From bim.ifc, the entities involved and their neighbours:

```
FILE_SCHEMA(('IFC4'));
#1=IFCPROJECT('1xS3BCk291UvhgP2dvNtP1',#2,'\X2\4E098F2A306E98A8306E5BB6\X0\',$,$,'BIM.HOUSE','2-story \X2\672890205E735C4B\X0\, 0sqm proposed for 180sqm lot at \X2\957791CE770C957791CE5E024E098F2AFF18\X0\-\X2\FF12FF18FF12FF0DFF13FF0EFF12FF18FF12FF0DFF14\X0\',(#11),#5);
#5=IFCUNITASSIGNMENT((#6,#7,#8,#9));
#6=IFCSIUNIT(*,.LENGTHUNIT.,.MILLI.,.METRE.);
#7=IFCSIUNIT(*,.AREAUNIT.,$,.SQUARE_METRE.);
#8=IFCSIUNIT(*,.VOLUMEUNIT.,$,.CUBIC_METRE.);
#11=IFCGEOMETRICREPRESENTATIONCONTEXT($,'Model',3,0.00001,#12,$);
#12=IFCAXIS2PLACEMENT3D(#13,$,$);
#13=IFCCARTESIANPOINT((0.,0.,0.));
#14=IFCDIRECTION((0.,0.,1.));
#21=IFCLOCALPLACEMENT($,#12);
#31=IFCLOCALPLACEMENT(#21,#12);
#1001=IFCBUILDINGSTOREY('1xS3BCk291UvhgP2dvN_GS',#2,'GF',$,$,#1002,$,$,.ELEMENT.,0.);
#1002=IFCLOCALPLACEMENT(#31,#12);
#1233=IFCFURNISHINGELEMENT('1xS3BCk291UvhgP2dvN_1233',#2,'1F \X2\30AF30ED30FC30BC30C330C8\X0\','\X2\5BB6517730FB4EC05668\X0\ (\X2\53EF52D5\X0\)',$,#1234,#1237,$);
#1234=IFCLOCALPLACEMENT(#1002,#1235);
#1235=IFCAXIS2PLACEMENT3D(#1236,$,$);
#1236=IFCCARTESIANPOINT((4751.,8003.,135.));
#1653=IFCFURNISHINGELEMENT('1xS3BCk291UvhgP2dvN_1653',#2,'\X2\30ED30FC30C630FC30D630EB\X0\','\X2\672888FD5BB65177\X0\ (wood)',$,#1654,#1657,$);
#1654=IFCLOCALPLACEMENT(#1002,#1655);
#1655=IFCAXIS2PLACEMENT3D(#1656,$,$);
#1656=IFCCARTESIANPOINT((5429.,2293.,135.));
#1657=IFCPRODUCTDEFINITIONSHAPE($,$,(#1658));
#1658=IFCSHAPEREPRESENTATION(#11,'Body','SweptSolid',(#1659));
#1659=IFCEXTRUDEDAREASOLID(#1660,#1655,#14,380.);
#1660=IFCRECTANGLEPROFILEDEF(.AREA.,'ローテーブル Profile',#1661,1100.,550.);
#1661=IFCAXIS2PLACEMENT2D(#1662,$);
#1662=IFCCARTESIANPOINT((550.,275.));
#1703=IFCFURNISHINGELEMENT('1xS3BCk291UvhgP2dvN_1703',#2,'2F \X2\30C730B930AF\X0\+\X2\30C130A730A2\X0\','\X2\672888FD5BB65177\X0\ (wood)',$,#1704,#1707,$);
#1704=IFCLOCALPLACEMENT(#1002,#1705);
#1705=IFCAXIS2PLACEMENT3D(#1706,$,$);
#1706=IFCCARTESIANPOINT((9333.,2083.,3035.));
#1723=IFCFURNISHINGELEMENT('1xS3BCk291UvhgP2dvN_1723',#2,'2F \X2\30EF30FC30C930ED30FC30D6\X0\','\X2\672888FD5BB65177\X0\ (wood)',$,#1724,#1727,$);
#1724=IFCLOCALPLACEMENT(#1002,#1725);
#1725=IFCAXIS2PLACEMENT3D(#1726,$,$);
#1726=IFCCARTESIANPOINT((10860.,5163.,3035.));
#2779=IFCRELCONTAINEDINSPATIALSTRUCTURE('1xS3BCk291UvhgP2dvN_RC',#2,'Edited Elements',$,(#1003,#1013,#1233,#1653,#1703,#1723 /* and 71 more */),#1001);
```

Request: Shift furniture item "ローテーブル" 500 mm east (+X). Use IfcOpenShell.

```python
import ifcopenshell
import ifcopenshell.api.geometry
import ifcopenshell.util.placement

model = ifcopenshell.open("bim.ifc")

item = model.by_guid("1xS3BCk291UvhgP2dvN_1653")
matrix = ifcopenshell.util.placement.get_local_placement(item.ObjectPlacement)
matrix[0, 3] += 500.0
ifcopenshell.api.geometry.edit_object_placement(model, product=item, matrix=matrix, is_si=False)

print(ifcopenshell.util.placement.get_local_placement(item.ObjectPlacement).round(3) + 0.0)

model.write("bim_edited.ifc")
```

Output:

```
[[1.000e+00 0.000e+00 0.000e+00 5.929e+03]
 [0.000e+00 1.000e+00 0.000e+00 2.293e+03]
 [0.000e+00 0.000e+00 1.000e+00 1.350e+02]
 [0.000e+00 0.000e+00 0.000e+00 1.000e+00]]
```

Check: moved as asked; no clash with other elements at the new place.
